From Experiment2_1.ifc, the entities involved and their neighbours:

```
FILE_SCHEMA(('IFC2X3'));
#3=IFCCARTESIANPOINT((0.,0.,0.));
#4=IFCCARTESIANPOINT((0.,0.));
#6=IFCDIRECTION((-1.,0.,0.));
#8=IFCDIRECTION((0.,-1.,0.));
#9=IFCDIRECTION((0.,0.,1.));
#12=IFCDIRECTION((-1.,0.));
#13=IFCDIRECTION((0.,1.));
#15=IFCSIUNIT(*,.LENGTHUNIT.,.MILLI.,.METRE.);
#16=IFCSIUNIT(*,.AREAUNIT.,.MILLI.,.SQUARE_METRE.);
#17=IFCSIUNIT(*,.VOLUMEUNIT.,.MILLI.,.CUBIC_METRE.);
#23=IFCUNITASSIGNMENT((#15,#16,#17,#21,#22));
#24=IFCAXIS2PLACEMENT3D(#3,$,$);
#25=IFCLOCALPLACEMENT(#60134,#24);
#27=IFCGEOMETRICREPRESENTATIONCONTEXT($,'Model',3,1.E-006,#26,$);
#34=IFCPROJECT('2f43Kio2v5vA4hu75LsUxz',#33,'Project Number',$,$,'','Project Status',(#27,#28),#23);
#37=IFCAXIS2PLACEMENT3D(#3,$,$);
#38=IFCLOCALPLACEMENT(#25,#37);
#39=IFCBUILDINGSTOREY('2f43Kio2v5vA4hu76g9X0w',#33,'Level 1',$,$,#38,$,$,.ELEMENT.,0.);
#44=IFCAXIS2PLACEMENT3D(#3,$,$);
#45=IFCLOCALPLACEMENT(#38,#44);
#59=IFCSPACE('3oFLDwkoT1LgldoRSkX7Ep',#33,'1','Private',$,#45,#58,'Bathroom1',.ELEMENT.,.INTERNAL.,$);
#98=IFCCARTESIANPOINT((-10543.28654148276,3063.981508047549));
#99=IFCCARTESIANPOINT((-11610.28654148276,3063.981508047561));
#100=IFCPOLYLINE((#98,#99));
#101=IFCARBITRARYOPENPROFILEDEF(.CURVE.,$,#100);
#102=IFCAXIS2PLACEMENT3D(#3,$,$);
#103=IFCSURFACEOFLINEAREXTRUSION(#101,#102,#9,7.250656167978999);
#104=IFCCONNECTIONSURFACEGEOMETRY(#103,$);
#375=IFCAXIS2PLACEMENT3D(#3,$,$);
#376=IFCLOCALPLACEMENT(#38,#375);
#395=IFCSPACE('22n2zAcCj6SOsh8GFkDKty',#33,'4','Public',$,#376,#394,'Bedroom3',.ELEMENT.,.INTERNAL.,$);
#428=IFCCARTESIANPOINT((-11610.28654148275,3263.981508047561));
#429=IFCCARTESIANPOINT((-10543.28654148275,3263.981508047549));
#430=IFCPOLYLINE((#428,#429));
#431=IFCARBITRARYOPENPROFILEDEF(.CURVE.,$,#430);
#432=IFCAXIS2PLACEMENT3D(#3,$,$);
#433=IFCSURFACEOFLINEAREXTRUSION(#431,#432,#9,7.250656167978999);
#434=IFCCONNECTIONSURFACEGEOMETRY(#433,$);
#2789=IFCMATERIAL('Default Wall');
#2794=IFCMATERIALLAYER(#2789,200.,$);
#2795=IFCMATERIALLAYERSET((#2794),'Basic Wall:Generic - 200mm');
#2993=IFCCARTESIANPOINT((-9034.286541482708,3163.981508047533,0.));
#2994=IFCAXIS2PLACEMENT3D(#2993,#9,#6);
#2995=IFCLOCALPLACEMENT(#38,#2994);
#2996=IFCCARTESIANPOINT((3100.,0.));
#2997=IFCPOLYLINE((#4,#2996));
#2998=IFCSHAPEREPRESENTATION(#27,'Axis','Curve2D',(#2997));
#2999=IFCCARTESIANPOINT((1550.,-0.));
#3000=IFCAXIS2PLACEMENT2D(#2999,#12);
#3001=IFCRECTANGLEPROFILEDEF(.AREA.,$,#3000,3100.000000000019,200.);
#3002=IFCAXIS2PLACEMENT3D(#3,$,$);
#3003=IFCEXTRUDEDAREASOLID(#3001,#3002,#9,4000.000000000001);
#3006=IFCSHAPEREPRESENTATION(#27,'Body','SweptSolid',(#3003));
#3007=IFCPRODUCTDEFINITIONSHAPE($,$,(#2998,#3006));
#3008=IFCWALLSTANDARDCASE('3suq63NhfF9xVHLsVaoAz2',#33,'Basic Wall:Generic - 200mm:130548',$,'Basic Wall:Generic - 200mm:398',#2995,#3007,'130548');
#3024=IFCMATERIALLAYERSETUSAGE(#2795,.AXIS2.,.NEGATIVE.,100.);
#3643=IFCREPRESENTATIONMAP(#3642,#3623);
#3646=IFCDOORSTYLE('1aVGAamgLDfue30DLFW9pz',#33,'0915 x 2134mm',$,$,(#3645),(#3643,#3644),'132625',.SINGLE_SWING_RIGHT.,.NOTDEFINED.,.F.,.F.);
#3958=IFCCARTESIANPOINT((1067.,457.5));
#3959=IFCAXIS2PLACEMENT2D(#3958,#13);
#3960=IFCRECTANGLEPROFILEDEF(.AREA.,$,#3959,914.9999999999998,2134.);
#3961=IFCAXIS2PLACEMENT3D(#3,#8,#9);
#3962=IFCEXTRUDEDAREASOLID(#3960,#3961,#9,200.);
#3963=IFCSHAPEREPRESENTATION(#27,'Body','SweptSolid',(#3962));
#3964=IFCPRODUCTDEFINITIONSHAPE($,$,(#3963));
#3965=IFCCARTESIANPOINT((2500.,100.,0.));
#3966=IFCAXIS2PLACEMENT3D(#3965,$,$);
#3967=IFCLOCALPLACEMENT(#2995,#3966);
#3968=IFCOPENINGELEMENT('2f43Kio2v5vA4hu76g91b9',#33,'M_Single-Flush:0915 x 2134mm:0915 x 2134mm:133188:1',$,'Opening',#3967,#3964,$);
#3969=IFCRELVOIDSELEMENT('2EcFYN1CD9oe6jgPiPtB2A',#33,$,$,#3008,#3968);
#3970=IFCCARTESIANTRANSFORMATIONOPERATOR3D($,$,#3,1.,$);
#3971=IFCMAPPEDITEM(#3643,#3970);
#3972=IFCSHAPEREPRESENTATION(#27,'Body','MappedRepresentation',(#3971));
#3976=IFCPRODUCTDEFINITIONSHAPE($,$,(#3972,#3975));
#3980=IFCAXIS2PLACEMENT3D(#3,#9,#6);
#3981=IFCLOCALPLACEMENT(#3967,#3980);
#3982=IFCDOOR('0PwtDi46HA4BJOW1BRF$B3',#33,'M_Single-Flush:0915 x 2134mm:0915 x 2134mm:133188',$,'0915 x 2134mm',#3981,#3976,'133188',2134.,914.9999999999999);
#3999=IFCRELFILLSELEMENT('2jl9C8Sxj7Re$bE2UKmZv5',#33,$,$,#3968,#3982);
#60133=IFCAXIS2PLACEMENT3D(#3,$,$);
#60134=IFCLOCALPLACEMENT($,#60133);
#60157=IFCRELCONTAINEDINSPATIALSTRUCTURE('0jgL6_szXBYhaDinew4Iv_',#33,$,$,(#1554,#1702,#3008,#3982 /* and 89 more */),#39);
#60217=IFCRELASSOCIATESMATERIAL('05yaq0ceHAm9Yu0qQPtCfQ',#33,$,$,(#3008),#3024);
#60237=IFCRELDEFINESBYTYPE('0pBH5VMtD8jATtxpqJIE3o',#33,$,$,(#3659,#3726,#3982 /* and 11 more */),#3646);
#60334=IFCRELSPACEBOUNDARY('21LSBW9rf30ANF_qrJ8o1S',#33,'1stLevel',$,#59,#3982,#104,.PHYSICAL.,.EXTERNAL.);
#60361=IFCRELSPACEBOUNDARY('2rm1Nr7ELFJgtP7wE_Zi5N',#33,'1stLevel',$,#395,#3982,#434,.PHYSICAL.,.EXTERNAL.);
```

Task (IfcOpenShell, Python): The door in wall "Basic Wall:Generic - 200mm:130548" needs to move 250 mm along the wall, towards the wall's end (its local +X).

```python
import numpy as np
import ifcopenshell
import ifcopenshell.api.geometry
import ifcopenshell.util.placement

model = ifcopenshell.open("Experiment2_1.ifc")

door = model.by_id(3982)
opening = door.FillsVoids[0].RelatingOpeningElement
wall = opening.VoidsElements[0].RelatingBuildingElement

wall_matrix = ifcopenshell.util.placement.get_local_placement(wall.ObjectPlacement)
shift = wall_matrix[:3, 0] * 250.0
before = ifcopenshell.util.placement.get_local_placement(door.ObjectPlacement)[:3, 3].copy()

# The door is placed relative to its opening, so it follows when the opening moves.
matrix = ifcopenshell.util.placement.get_local_placement(opening.ObjectPlacement)
matrix[:3, 3] += shift
ifcopenshell.api.geometry.edit_object_placement(
    model, product=opening, matrix=matrix, is_si=False, should_transform_children=True
)

# Space boundary surfaces are stored in each space's coordinates; move them too.
for rel in door.ProvidesBoundaries:
    if not rel.ConnectionGeometry:
        continue
    surface = rel.ConnectionGeometry.SurfaceOnRelatingElement
    space_matrix = ifcopenshell.util.placement.get_local_placement(rel.RelatingSpace.ObjectPlacement)
    point = np.array(surface.Position.Location.Coordinates) + space_matrix[:3, :3].T @ shift
    surface.Position = model.createIfcAxis2Placement3D(
        model.createIfcCartesianPoint(point.tolist()), surface.Position.Axis, surface.Position.RefDirection
    )

after = ifcopenshell.util.placement.get_local_placement(door.ObjectPlacement)[:3, 3]
print("door moved by", (after - before).round(3) + 0.0)

model.write("Experiment2_1_v2.ifc")
```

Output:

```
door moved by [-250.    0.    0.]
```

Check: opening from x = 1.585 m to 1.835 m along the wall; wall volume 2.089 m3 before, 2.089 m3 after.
